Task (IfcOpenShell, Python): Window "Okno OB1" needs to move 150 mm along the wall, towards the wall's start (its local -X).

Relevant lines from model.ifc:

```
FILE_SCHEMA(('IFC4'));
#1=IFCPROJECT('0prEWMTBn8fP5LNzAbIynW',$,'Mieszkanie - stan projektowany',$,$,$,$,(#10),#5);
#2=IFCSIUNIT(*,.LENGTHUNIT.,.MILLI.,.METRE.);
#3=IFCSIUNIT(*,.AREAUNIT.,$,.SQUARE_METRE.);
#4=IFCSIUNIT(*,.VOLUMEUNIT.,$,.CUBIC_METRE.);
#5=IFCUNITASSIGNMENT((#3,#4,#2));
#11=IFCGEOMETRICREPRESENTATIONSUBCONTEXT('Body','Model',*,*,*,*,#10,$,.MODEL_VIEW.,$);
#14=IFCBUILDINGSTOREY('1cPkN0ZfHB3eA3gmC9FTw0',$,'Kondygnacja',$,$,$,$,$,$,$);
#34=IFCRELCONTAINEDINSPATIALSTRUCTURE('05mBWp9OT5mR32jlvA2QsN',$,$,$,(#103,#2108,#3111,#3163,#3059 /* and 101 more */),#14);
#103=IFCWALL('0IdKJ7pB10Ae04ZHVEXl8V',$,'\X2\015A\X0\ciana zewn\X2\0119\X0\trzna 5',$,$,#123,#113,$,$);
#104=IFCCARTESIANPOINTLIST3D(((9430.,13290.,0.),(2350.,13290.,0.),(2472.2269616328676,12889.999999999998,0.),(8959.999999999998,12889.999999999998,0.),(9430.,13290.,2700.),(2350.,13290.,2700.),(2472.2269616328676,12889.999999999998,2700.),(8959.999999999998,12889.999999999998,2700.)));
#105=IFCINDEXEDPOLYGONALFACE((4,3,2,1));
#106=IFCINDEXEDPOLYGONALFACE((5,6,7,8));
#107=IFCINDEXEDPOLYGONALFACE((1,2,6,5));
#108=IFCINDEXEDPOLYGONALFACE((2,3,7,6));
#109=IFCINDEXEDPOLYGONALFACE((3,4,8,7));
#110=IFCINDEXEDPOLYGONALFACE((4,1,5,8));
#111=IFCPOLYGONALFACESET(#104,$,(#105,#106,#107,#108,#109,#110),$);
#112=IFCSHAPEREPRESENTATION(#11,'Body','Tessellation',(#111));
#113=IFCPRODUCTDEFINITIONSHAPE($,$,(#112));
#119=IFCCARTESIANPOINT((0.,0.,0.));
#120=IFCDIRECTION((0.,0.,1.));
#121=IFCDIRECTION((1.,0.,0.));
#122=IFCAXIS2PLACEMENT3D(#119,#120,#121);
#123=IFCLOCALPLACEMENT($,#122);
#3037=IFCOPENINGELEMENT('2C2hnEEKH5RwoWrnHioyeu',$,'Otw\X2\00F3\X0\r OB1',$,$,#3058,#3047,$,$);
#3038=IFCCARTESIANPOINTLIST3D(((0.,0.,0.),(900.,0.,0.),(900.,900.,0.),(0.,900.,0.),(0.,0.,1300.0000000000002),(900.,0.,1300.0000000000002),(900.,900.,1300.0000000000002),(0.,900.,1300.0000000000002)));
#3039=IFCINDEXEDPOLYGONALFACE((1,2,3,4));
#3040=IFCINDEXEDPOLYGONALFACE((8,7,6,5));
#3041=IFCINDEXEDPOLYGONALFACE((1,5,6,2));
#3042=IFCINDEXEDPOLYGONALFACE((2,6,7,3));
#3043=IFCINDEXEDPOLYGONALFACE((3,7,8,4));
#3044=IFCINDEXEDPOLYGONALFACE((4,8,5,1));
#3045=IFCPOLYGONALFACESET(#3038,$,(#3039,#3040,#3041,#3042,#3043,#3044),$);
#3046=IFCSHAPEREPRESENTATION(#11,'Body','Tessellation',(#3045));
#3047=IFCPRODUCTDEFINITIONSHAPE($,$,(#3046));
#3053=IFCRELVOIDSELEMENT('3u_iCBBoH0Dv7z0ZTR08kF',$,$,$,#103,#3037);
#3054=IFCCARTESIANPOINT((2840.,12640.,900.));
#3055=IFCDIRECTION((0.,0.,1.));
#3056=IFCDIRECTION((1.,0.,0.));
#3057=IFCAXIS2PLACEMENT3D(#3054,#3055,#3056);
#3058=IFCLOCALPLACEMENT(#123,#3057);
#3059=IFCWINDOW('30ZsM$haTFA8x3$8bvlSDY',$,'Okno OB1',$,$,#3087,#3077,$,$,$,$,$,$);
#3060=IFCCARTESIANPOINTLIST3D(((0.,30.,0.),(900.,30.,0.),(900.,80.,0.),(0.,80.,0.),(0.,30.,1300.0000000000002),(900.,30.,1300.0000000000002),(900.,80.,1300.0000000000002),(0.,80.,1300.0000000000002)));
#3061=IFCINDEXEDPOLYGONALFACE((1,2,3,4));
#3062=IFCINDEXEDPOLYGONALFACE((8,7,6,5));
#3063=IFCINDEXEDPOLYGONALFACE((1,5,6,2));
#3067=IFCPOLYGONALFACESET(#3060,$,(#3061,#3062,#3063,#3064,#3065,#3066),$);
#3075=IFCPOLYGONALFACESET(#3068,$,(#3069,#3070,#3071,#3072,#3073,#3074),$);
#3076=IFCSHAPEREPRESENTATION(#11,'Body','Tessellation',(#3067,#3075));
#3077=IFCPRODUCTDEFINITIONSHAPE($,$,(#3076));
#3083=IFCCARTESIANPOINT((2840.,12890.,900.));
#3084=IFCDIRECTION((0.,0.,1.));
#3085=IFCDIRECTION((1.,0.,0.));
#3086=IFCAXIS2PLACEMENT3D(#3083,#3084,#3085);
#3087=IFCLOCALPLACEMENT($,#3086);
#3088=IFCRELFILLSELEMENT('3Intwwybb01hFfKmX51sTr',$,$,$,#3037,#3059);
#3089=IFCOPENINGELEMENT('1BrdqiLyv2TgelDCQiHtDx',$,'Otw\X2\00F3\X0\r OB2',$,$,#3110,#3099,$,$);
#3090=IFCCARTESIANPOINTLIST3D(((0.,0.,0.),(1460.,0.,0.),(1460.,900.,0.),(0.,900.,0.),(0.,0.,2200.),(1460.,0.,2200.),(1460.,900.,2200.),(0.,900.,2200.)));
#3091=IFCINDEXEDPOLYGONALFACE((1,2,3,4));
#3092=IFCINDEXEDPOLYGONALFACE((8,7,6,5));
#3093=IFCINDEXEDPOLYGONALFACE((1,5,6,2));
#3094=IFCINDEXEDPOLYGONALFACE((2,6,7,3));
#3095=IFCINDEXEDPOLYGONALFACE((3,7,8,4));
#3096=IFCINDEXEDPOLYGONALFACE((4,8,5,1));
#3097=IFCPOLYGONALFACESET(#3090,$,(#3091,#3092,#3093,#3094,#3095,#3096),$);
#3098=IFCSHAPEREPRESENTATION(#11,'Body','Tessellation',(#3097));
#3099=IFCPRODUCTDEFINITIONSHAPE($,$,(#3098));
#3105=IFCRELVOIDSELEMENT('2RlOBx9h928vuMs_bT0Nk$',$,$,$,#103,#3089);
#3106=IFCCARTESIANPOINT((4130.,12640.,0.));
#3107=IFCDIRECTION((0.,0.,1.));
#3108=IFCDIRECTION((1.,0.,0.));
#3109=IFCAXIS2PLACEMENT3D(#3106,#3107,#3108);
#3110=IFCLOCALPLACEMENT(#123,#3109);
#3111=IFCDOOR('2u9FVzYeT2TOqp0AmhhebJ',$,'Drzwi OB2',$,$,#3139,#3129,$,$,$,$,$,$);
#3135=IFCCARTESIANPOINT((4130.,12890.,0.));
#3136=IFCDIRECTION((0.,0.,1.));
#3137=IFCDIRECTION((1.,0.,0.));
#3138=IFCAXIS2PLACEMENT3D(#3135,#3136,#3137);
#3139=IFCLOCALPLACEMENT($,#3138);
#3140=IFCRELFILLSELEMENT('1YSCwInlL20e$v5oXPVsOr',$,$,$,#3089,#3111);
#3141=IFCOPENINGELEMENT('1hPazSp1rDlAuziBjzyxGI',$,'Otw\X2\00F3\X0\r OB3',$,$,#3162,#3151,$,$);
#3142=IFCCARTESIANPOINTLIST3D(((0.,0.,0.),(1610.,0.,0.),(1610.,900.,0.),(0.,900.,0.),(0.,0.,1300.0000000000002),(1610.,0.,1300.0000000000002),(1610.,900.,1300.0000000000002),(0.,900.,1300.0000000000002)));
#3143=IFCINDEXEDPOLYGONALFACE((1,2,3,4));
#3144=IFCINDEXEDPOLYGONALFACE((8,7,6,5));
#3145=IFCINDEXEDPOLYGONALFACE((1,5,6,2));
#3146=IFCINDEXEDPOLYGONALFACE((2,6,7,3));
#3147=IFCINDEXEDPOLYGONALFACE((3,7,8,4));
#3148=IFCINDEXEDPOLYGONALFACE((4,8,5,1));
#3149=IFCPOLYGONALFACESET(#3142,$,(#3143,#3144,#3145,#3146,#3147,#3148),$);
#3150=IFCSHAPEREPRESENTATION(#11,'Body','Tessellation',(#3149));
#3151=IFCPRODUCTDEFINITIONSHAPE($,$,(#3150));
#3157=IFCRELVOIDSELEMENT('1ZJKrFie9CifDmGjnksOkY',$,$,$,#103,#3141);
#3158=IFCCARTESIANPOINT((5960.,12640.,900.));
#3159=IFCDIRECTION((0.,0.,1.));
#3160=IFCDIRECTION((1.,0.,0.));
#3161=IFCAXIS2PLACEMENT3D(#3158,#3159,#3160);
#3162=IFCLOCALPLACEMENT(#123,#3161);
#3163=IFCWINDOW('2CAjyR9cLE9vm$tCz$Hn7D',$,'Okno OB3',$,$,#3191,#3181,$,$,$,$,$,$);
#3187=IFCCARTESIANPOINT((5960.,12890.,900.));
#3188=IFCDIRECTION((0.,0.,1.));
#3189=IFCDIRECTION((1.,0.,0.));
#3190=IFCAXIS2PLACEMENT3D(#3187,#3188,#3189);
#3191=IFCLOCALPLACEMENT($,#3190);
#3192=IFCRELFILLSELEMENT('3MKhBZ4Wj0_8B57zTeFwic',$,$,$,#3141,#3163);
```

```python
import ifcopenshell
import ifcopenshell.api.geometry
import ifcopenshell.util.placement
import ifcopenshell.util.unit

model = ifcopenshell.open("model.ifc")
unit_scale = ifcopenshell.util.unit.calculate_unit_scale(model)

window = model.by_guid("30ZsM$haTFA8x3$8bvlSDY")
opening = window.FillsVoids[0].RelatingOpeningElement
wall = opening.VoidsElements[0].RelatingBuildingElement

wall_matrix = ifcopenshell.util.placement.get_local_placement(wall.ObjectPlacement)
shift = wall_matrix[:3, 0] * -0.15 / unit_scale
before = ifcopenshell.util.placement.get_local_placement(window.ObjectPlacement)[:3, 3].copy()

# The window is not placed relative to its opening, so move both.
for product in (opening, window):
    matrix = ifcopenshell.util.placement.get_local_placement(product.ObjectPlacement)
    matrix[:3, 3] += shift
    ifcopenshell.api.geometry.edit_object_placement(model, product=product, matrix=matrix, is_si=False)

after = ifcopenshell.util.placement.get_local_placement(window.ObjectPlacement)[:3, 3]
print("window moved by", (after - before).round(3) + 0.0)

model.write("model_edited.ifc")
```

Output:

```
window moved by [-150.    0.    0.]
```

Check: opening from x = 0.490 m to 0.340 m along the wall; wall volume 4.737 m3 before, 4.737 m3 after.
